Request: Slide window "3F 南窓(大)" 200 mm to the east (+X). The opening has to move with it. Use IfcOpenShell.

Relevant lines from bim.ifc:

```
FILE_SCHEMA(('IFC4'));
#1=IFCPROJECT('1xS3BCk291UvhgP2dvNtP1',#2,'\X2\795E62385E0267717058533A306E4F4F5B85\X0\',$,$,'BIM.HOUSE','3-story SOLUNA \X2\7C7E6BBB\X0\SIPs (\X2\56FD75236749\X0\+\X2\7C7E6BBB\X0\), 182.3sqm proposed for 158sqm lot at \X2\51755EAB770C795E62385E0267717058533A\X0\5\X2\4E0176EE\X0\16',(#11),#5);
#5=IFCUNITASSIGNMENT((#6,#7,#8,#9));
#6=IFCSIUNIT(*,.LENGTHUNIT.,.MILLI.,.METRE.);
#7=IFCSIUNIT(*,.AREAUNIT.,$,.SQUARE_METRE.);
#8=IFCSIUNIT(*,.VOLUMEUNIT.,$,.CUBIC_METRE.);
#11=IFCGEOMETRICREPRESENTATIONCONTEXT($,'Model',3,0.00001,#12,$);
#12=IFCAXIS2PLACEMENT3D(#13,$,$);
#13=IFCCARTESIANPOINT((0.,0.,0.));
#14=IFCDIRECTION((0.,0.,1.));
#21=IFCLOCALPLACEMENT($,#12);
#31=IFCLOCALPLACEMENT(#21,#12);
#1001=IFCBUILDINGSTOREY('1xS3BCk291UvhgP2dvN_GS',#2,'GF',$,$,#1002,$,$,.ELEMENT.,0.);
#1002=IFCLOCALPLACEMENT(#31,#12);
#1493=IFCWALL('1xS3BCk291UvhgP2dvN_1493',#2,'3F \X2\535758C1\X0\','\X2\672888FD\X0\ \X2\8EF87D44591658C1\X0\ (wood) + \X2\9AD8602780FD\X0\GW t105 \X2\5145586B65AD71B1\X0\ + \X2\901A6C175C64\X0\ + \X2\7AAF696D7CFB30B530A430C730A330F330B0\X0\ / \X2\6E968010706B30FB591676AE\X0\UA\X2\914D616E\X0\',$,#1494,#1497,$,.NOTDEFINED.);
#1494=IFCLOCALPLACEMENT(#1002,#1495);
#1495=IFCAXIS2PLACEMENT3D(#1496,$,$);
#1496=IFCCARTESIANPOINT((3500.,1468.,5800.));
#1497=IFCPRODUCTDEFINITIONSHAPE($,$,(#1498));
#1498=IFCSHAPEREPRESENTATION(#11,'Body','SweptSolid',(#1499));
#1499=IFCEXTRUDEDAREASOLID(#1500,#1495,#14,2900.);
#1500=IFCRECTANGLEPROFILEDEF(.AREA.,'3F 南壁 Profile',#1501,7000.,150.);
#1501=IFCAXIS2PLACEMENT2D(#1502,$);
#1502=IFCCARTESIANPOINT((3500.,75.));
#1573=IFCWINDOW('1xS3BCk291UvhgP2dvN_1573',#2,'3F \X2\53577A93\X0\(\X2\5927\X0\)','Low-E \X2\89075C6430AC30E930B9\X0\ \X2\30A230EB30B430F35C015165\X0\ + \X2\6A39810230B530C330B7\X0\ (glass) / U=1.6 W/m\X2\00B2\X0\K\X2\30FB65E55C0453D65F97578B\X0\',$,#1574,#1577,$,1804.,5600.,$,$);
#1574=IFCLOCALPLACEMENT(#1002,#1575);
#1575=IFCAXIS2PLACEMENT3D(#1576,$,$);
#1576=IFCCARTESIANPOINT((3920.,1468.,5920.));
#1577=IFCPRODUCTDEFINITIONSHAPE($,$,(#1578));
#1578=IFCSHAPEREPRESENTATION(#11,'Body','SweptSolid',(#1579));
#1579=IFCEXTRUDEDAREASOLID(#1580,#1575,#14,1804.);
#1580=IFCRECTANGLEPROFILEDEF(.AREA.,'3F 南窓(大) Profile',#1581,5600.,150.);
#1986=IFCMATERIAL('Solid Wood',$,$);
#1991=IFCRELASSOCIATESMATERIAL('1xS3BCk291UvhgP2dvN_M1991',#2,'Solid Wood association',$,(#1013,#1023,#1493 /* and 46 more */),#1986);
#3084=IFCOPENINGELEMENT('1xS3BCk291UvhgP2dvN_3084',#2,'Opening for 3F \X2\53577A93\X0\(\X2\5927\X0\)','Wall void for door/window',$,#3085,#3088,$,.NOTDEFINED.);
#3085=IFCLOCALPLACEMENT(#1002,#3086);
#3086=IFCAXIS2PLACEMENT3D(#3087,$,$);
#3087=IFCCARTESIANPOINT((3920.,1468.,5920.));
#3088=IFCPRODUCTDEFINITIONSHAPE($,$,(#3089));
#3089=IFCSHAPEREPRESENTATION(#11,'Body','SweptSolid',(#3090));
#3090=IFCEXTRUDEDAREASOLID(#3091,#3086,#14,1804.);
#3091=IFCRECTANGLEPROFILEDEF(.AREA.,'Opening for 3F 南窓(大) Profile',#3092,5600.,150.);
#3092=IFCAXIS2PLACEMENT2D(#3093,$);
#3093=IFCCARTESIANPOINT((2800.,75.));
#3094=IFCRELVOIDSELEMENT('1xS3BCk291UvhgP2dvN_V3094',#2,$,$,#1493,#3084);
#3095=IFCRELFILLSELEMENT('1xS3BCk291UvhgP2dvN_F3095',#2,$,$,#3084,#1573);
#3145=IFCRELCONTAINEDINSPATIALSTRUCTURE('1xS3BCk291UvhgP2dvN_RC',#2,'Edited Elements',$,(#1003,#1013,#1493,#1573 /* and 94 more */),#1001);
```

```python
import ifcopenshell
import ifcopenshell.api.geometry
import ifcopenshell.util.placement

model = ifcopenshell.open("bim.ifc")

window = model.by_guid("1xS3BCk291UvhgP2dvN_1573")
opening = window.FillsVoids[0].RelatingOpeningElement
wall = opening.VoidsElements[0].RelatingBuildingElement

wall_matrix = ifcopenshell.util.placement.get_local_placement(wall.ObjectPlacement)
shift = wall_matrix[:3, 0] * 200.0
before = ifcopenshell.util.placement.get_local_placement(window.ObjectPlacement)[:3, 3].copy()

# The window is not placed relative to its opening, so move both.
for product in (opening, window):
    matrix = ifcopenshell.util.placement.get_local_placement(product.ObjectPlacement)
    matrix[:3, 3] += shift
    ifcopenshell.api.geometry.edit_object_placement(model, product=product, matrix=matrix, is_si=False)

after = ifcopenshell.util.placement.get_local_placement(window.ObjectPlacement)[:3, 3]
print("window moved by", (after - before).round(3) + 0.0)

model.write("bim_v2.ifc")
```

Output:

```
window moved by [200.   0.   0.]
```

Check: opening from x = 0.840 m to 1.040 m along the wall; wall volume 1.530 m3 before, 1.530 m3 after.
